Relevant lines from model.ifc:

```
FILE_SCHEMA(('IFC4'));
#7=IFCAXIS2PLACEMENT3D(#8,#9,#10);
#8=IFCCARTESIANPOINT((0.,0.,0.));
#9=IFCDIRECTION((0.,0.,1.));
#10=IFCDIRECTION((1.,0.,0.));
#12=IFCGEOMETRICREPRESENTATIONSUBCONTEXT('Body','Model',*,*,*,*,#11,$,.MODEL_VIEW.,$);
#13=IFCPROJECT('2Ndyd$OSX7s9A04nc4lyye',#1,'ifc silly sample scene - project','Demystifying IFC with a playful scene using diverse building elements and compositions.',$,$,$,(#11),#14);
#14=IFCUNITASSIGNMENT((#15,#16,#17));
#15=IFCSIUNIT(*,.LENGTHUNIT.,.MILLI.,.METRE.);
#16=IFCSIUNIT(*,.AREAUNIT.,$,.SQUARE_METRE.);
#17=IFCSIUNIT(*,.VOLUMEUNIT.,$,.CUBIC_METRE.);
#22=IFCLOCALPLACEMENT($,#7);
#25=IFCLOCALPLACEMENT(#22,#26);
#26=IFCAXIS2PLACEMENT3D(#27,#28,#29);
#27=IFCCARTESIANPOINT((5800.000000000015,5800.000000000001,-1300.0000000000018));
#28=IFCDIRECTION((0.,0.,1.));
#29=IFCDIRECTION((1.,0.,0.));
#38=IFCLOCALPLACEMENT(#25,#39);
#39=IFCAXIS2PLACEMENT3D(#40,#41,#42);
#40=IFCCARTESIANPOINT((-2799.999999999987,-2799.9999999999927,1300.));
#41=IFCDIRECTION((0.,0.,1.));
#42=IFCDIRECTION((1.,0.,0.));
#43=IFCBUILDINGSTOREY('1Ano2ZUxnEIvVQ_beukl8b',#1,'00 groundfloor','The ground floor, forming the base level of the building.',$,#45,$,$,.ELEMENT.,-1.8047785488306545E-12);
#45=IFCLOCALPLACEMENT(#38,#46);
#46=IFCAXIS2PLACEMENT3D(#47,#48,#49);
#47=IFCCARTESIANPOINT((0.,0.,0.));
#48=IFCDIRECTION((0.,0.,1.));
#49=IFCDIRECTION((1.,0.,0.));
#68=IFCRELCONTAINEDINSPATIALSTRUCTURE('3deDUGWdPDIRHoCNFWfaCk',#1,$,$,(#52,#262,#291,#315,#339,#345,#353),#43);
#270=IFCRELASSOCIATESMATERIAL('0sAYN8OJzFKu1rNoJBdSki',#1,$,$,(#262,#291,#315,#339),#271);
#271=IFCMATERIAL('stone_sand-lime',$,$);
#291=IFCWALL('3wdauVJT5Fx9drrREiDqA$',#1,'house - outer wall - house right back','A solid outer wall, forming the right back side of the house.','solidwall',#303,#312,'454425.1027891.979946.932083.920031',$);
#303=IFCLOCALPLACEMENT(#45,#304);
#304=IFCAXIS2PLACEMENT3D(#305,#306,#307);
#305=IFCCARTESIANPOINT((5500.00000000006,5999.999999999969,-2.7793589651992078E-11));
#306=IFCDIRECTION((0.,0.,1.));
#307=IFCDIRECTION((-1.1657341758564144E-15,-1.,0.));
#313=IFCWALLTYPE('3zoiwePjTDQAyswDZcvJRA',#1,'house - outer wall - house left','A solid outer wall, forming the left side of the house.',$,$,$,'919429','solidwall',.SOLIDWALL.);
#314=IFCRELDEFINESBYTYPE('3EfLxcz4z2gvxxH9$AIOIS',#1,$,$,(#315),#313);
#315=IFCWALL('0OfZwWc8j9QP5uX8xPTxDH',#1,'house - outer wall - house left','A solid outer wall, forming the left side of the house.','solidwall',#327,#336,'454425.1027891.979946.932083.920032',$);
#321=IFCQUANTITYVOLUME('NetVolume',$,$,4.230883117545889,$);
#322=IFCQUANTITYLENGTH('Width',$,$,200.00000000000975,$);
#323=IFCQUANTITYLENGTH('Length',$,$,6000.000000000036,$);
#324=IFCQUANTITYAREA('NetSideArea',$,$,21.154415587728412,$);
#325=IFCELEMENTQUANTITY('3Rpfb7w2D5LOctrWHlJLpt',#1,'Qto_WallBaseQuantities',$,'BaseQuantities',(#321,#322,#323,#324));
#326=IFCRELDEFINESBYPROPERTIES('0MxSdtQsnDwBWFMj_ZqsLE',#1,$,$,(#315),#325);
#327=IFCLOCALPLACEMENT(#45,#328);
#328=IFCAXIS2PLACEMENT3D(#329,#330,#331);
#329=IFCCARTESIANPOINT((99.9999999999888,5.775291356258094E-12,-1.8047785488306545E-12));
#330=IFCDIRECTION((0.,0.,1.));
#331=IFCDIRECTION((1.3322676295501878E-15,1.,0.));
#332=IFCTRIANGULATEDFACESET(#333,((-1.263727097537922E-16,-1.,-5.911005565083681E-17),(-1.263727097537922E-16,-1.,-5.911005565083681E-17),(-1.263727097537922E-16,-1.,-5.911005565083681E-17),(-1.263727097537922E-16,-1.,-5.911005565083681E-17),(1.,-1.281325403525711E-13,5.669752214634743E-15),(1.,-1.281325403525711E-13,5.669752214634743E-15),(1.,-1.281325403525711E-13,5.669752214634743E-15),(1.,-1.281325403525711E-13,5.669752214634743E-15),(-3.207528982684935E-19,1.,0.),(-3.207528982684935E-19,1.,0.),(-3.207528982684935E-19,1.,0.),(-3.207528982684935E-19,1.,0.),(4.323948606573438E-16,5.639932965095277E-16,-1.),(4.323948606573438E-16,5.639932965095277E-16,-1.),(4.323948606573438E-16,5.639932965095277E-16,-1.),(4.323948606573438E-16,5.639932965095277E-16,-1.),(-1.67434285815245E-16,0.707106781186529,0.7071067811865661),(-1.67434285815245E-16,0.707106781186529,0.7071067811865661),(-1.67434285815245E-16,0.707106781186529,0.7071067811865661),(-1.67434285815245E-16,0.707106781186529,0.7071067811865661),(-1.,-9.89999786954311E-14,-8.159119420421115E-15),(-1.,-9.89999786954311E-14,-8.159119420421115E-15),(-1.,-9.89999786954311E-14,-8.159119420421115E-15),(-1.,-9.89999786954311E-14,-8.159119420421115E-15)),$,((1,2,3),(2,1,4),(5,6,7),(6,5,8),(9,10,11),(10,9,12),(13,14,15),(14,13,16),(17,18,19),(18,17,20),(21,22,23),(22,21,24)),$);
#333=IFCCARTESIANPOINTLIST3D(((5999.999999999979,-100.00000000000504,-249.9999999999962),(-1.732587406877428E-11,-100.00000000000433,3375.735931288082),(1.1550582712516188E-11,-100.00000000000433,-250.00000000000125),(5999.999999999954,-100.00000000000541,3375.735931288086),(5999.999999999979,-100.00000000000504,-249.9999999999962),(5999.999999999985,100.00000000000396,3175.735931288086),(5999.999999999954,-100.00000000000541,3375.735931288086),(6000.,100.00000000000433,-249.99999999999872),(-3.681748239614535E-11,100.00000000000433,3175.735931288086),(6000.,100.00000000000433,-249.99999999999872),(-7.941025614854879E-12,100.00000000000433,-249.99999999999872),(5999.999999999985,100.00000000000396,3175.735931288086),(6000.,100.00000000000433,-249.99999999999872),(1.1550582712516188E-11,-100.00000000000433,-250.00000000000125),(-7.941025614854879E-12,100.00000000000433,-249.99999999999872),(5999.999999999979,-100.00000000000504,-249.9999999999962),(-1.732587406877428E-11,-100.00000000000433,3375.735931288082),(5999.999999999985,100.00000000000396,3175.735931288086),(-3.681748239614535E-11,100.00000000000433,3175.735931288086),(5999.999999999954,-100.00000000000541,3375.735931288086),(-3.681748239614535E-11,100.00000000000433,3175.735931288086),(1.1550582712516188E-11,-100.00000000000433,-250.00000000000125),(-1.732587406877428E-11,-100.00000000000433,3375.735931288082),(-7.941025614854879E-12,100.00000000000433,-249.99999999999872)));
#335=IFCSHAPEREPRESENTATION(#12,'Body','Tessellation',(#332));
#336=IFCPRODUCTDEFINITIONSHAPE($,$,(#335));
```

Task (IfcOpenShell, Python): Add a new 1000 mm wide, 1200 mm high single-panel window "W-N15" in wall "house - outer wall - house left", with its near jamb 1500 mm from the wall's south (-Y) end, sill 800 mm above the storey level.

```python
import numpy as np
import ifcopenshell
import ifcopenshell.api.feature
import ifcopenshell.api.geometry
import ifcopenshell.api.pset
import ifcopenshell.api.root
import ifcopenshell.api.spatial
import ifcopenshell.geom
import ifcopenshell.util.element
import ifcopenshell.util.placement
import ifcopenshell.util.representation
import ifcopenshell.util.shape
import ifcopenshell.util.unit

model = ifcopenshell.open("model.ifc")
unit_scale = ifcopenshell.util.unit.calculate_unit_scale(model)
area_scale = ifcopenshell.util.unit.calculate_unit_scale(model, "AREAUNIT")
volume_scale = ifcopenshell.util.unit.calculate_unit_scale(model, "VOLUMEUNIT")
settings = ifcopenshell.geom.settings()


def volume(element):
    """Net volume in cubic metres, openings subtracted."""
    shape = ifcopenshell.geom.create_shape(settings, element)
    return ifcopenshell.util.shape.get_volume(shape.geometry)


wall = model.by_guid("0OfZwWc8j9QP5uX8xPTxDH")
storey = ifcopenshell.util.element.get_container(wall, ifc_class="IfcBuildingStorey")
context = ifcopenshell.util.representation.get_context(model, "Model", "Body", "MODEL_VIEW")
before = volume(wall)

width, height, from_end, sill = 1, 1.2, 1.5, 0.8  # metres

# The wall runs along its own X axis, and the end named is its -X end.
wall_shape = ifcopenshell.geom.create_shape(settings, wall)
x, y, z = ifcopenshell.util.shape.get_vertices(wall_shape.geometry).T
start = x.min() + from_end
face, thickness = float(y.min()), float(y.max() - y.min())
wall_matrix = ifcopenshell.util.placement.get_local_placement(wall.ObjectPlacement)
level = ifcopenshell.util.placement.get_local_placement(storey.ObjectPlacement)[2, 3]


def in_wall(x, y):
    """Placement at x, y metres in the wall's axes, at sill height."""
    matrix = wall_matrix.copy()
    matrix[:, 3] = wall_matrix @ np.array([x / unit_scale, y / unit_scale, 0.0, 1.0])
    matrix[2, 3] = level + sill / unit_scale
    return matrix


# Opening: a box that overshoots both wall faces by 50 mm.
opening = ifcopenshell.api.root.create_entity(model, ifc_class="IfcOpeningElement", predefined_type="OPENING")
box = ifcopenshell.api.geometry.add_wall_representation(
    model, context=context, length=width, height=height, thickness=thickness + 0.1
)
ifcopenshell.api.geometry.assign_representation(model, product=opening, representation=box)
ifcopenshell.api.geometry.edit_object_placement(model, product=opening, matrix=in_wall(start, face - 0.05), is_si=False)
ifcopenshell.api.feature.add_feature(model, feature=opening, element=wall)

window = ifcopenshell.api.root.create_entity(model, ifc_class="IfcWindow", name="W-N15", predefined_type="WINDOW")
window.OverallWidth, window.OverallHeight = width / unit_scale, height / unit_scale
window.PartitioningType = "SINGLE_PANEL"
body = ifcopenshell.api.geometry.add_window_representation(
    model,
    context=context,
    overall_width=window.OverallWidth,
    overall_height=window.OverallHeight,
    partition_type="SINGLE_PANEL",
)
ifcopenshell.api.geometry.assign_representation(model, product=window, representation=body)
ifcopenshell.api.spatial.assign_container(model, products=[window], relating_structure=storey)
ifcopenshell.api.feature.add_filling(model, opening=opening, element=window)

# Centre the window in the wall's thickness.
ifcopenshell.api.geometry.edit_object_placement(model, product=window, matrix=in_wall(start, face), is_si=False)
window_shape = ifcopenshell.geom.create_shape(settings, window)
depth = ifcopenshell.util.shape.get_vertices(window_shape.geometry)[:, 1]
offset = face + thickness / 2 - (depth.min() + depth.max()) / 2
ifcopenshell.api.geometry.edit_object_placement(model, product=window, matrix=in_wall(start, offset), is_si=False)

after = volume(wall)

# Update the wall's stored quantities.
qto = model.by_id(ifcopenshell.util.element.get_pset(wall, "Qto_WallBaseQuantities", should_inherit=False)["id"])
ifcopenshell.api.pset.edit_qto(model, qto=qto, properties={
    "NetVolume": after / volume_scale,
    "NetSideArea": after / thickness / area_scale,
})

print(f"wall volume {before:.3f} -> {after:.3f} m3")

model.write("model_edited.ifc")
```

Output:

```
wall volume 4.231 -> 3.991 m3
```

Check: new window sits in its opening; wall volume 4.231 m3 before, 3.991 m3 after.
